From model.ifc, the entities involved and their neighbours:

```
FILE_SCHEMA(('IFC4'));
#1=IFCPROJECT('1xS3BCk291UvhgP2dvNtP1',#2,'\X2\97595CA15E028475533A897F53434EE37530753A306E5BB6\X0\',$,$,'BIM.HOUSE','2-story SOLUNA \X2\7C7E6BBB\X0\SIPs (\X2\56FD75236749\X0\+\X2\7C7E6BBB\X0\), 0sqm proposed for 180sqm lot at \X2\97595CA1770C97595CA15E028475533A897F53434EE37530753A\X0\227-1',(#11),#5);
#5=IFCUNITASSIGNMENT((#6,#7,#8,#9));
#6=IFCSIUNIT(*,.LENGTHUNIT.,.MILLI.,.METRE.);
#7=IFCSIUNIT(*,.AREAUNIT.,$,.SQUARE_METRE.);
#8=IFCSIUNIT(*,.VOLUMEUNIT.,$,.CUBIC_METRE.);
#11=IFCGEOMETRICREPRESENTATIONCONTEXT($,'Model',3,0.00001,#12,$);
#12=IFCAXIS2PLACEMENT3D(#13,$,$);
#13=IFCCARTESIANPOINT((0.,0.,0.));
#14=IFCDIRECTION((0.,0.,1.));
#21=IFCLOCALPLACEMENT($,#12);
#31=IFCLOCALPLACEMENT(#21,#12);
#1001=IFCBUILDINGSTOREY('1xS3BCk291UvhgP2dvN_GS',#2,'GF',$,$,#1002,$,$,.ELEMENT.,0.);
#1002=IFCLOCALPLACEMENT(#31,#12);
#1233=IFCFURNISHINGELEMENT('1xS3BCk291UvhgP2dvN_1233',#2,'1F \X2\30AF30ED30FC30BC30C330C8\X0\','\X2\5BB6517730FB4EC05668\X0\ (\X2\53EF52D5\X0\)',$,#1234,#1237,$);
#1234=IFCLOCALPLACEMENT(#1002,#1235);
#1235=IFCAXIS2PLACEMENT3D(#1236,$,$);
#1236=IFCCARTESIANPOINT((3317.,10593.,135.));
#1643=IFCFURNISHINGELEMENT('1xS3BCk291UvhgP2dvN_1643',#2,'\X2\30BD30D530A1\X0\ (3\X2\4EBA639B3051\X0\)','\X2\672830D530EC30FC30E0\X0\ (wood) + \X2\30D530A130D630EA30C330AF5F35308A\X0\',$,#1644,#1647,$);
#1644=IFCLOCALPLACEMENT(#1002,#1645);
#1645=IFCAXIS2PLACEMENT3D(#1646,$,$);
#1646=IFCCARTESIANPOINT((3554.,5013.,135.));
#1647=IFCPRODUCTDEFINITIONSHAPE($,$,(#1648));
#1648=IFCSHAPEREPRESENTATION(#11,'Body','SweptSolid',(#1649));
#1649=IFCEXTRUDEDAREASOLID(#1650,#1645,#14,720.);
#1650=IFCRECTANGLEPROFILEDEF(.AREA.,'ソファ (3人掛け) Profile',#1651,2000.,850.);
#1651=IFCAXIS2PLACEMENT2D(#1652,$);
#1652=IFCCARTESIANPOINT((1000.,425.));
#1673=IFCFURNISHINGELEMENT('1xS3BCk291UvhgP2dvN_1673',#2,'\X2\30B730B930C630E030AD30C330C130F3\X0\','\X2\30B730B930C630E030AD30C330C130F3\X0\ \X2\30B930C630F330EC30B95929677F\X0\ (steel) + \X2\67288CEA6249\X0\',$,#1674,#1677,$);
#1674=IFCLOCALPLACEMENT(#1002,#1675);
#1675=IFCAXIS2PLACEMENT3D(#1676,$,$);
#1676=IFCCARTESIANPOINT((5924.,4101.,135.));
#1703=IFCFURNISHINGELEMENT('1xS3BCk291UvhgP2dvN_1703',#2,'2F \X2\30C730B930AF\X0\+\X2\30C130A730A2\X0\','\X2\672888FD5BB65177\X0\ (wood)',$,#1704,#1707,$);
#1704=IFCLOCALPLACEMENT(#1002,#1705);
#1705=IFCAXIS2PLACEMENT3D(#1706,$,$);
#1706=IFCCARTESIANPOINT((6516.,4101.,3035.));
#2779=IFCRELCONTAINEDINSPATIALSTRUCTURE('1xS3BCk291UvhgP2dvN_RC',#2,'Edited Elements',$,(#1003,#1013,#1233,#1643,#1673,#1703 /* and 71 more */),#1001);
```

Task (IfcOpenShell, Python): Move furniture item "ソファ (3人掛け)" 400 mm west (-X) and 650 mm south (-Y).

```python
import ifcopenshell
import ifcopenshell.api.geometry
import ifcopenshell.util.placement

model = ifcopenshell.open("model.ifc")

item = model.by_guid("1xS3BCk291UvhgP2dvN_1643")
matrix = ifcopenshell.util.placement.get_local_placement(item.ObjectPlacement)
matrix[0, 3] -= 400.0
matrix[1, 3] -= 650.0
ifcopenshell.api.geometry.edit_object_placement(model, product=item, matrix=matrix, is_si=False)

print(ifcopenshell.util.placement.get_local_placement(item.ObjectPlacement).round(3) + 0.0)

model.write("model-out.ifc")
```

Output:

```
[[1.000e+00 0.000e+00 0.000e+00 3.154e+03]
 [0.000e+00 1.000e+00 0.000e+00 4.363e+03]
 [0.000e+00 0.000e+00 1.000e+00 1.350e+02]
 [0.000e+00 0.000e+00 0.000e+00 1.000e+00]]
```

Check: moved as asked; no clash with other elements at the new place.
